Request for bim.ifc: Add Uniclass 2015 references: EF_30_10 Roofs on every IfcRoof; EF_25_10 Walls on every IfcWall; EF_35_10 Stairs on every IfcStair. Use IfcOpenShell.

First a look at what the model holds.

```python
import ifcopenshell

model = ifcopenshell.open("bim.ifc")
print(model.schema)
print("classifications:", [c.Name for c in model.by_type("IfcClassification")])
for ifc_class in ("IfcDoor", "IfcRoof", "IfcStair", "IfcWall", "IfcWindow"):
    print(ifc_class, len(model.by_type(ifc_class)))
```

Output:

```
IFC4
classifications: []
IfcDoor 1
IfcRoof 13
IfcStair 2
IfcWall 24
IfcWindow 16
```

```python
import ifcopenshell
import ifcopenshell.api.classification

model = ifcopenshell.open("bim.ifc")

system = ifcopenshell.api.classification.add_classification(model, classification="Uniclass 2015")

codes = {
    "IfcRoof": ("EF_30_10", "Roofs"),
    "IfcWall": ("EF_25_10", "Walls"),
    "IfcStair": ("EF_35_10", "Stairs"),
}
for ifc_class, (code, name) in codes.items():
    products = model.by_type(ifc_class)
    ifcopenshell.api.classification.add_reference(
        model, products=products, classification=system, identification=code, name=name
    )
    print(code, len(products))

model.write("bim_edited.ifc")
```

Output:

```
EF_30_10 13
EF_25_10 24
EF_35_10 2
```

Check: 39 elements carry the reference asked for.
